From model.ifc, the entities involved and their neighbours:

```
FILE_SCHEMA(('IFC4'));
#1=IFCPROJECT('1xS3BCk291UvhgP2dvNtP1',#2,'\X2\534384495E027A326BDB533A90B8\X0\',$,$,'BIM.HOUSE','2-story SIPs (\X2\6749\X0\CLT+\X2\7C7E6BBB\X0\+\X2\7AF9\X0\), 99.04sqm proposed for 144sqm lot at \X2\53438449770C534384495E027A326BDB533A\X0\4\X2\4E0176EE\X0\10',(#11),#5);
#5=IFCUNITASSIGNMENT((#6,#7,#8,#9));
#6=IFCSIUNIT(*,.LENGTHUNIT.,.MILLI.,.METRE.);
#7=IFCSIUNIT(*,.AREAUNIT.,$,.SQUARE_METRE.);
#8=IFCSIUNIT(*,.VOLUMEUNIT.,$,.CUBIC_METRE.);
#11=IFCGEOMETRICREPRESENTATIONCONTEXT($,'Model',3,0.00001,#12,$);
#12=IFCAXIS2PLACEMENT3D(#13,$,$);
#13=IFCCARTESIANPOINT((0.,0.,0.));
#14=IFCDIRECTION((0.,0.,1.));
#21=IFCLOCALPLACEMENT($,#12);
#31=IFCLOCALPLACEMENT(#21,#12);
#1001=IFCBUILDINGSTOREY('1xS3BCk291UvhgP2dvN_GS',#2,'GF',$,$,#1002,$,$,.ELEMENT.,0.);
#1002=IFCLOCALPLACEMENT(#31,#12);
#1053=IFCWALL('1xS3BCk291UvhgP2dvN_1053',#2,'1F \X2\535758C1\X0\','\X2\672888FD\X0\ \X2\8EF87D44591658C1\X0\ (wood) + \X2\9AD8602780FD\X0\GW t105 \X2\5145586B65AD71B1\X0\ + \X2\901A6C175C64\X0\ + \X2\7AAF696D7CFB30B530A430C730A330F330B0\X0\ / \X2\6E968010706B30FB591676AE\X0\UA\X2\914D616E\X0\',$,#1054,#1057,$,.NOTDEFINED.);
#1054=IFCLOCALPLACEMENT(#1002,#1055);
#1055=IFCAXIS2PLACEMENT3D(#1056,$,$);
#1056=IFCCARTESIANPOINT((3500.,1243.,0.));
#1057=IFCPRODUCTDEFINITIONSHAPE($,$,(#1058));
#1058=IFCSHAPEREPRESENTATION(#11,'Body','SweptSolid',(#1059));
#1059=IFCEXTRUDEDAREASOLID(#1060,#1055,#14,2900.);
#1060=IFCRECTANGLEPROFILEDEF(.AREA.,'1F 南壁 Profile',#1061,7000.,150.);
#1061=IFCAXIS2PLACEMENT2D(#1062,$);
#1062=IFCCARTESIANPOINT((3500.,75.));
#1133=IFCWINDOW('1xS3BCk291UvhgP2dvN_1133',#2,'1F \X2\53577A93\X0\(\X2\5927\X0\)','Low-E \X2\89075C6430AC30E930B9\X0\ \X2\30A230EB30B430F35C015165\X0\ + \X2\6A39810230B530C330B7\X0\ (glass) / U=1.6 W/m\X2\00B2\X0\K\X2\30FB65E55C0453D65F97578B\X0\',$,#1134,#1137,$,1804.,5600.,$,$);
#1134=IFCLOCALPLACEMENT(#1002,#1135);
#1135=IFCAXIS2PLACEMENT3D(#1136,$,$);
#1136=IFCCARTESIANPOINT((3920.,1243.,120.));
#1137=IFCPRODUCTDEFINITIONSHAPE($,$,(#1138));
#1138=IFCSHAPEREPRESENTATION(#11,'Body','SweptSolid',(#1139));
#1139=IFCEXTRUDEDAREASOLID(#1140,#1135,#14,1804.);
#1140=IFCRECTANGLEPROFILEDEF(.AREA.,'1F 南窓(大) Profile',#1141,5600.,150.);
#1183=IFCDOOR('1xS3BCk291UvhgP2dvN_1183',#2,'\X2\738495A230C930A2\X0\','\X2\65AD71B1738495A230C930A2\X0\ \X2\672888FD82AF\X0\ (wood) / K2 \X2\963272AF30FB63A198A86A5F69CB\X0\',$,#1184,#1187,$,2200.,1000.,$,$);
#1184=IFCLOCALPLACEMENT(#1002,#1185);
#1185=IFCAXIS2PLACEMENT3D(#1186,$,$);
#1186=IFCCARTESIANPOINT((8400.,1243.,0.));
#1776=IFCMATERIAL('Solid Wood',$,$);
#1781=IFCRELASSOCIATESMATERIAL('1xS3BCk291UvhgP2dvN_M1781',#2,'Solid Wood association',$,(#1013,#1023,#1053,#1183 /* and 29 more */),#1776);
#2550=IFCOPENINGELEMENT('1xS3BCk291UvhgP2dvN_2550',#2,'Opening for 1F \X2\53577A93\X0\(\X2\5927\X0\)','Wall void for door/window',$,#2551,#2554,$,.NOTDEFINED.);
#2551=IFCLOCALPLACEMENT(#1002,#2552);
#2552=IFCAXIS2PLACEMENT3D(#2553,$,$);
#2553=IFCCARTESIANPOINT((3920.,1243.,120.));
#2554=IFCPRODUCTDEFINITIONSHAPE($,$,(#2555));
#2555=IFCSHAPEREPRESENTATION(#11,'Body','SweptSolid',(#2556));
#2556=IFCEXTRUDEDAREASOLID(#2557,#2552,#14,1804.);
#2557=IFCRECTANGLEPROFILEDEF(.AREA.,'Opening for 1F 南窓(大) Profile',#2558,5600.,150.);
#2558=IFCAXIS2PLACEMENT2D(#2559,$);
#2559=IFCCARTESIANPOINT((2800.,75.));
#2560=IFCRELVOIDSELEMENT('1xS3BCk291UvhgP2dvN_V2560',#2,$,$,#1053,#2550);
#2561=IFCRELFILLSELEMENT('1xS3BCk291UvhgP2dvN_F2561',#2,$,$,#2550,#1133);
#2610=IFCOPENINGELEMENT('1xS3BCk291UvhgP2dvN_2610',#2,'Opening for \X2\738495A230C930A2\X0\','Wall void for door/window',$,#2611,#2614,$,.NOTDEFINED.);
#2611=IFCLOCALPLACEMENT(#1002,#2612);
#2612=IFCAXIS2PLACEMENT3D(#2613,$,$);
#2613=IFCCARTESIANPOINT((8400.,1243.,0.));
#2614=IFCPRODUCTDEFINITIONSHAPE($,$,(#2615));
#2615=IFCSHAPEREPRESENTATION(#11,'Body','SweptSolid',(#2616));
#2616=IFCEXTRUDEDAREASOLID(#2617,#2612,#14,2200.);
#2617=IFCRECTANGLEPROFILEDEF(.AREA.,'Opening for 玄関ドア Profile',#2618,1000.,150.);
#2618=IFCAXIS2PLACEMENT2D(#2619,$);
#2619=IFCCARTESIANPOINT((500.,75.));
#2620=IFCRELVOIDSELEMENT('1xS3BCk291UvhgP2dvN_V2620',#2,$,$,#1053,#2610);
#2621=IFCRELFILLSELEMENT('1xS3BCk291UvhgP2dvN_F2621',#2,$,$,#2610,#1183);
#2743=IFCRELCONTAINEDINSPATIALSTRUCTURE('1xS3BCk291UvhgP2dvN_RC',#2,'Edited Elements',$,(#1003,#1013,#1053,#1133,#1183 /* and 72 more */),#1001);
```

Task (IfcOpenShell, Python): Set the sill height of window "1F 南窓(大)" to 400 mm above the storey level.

```python
import numpy as np
import ifcopenshell
import ifcopenshell.api.geometry
import ifcopenshell.geom
import ifcopenshell.util.element
import ifcopenshell.util.placement
import ifcopenshell.util.shape
import ifcopenshell.util.unit

model = ifcopenshell.open("model.ifc")
unit_scale = ifcopenshell.util.unit.calculate_unit_scale(model)

window = model.by_id(1133)
opening = window.FillsVoids[0].RelatingOpeningElement
storey = ifcopenshell.util.element.get_container(window, ifc_class="IfcBuildingStorey")
level = ifcopenshell.util.placement.get_local_placement(storey.ObjectPlacement)[2, 3]

# The opening's origin need not be at the sill, so measure its lowest point.
shape = ifcopenshell.geom.create_shape(ifcopenshell.geom.settings(), opening)
bottom = ifcopenshell.util.shape.get_shape_bottom_elevation(shape, shape.geometry) / unit_scale
dz = level + 0.4 / unit_scale - bottom

shift = np.array([0.0, 0.0, dz])
# The window is not placed relative to its opening, so move both.
for product in (opening, window):
    matrix = ifcopenshell.util.placement.get_local_placement(product.ObjectPlacement)
    matrix[:3, 3] += shift
    ifcopenshell.api.geometry.edit_object_placement(model, product=product, matrix=matrix, is_si=False)

print(f"moved by {dz * unit_scale:+.3f} m")

model.write("model_rev.ifc")
```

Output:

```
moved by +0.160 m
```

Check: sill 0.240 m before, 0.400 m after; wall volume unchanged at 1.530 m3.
